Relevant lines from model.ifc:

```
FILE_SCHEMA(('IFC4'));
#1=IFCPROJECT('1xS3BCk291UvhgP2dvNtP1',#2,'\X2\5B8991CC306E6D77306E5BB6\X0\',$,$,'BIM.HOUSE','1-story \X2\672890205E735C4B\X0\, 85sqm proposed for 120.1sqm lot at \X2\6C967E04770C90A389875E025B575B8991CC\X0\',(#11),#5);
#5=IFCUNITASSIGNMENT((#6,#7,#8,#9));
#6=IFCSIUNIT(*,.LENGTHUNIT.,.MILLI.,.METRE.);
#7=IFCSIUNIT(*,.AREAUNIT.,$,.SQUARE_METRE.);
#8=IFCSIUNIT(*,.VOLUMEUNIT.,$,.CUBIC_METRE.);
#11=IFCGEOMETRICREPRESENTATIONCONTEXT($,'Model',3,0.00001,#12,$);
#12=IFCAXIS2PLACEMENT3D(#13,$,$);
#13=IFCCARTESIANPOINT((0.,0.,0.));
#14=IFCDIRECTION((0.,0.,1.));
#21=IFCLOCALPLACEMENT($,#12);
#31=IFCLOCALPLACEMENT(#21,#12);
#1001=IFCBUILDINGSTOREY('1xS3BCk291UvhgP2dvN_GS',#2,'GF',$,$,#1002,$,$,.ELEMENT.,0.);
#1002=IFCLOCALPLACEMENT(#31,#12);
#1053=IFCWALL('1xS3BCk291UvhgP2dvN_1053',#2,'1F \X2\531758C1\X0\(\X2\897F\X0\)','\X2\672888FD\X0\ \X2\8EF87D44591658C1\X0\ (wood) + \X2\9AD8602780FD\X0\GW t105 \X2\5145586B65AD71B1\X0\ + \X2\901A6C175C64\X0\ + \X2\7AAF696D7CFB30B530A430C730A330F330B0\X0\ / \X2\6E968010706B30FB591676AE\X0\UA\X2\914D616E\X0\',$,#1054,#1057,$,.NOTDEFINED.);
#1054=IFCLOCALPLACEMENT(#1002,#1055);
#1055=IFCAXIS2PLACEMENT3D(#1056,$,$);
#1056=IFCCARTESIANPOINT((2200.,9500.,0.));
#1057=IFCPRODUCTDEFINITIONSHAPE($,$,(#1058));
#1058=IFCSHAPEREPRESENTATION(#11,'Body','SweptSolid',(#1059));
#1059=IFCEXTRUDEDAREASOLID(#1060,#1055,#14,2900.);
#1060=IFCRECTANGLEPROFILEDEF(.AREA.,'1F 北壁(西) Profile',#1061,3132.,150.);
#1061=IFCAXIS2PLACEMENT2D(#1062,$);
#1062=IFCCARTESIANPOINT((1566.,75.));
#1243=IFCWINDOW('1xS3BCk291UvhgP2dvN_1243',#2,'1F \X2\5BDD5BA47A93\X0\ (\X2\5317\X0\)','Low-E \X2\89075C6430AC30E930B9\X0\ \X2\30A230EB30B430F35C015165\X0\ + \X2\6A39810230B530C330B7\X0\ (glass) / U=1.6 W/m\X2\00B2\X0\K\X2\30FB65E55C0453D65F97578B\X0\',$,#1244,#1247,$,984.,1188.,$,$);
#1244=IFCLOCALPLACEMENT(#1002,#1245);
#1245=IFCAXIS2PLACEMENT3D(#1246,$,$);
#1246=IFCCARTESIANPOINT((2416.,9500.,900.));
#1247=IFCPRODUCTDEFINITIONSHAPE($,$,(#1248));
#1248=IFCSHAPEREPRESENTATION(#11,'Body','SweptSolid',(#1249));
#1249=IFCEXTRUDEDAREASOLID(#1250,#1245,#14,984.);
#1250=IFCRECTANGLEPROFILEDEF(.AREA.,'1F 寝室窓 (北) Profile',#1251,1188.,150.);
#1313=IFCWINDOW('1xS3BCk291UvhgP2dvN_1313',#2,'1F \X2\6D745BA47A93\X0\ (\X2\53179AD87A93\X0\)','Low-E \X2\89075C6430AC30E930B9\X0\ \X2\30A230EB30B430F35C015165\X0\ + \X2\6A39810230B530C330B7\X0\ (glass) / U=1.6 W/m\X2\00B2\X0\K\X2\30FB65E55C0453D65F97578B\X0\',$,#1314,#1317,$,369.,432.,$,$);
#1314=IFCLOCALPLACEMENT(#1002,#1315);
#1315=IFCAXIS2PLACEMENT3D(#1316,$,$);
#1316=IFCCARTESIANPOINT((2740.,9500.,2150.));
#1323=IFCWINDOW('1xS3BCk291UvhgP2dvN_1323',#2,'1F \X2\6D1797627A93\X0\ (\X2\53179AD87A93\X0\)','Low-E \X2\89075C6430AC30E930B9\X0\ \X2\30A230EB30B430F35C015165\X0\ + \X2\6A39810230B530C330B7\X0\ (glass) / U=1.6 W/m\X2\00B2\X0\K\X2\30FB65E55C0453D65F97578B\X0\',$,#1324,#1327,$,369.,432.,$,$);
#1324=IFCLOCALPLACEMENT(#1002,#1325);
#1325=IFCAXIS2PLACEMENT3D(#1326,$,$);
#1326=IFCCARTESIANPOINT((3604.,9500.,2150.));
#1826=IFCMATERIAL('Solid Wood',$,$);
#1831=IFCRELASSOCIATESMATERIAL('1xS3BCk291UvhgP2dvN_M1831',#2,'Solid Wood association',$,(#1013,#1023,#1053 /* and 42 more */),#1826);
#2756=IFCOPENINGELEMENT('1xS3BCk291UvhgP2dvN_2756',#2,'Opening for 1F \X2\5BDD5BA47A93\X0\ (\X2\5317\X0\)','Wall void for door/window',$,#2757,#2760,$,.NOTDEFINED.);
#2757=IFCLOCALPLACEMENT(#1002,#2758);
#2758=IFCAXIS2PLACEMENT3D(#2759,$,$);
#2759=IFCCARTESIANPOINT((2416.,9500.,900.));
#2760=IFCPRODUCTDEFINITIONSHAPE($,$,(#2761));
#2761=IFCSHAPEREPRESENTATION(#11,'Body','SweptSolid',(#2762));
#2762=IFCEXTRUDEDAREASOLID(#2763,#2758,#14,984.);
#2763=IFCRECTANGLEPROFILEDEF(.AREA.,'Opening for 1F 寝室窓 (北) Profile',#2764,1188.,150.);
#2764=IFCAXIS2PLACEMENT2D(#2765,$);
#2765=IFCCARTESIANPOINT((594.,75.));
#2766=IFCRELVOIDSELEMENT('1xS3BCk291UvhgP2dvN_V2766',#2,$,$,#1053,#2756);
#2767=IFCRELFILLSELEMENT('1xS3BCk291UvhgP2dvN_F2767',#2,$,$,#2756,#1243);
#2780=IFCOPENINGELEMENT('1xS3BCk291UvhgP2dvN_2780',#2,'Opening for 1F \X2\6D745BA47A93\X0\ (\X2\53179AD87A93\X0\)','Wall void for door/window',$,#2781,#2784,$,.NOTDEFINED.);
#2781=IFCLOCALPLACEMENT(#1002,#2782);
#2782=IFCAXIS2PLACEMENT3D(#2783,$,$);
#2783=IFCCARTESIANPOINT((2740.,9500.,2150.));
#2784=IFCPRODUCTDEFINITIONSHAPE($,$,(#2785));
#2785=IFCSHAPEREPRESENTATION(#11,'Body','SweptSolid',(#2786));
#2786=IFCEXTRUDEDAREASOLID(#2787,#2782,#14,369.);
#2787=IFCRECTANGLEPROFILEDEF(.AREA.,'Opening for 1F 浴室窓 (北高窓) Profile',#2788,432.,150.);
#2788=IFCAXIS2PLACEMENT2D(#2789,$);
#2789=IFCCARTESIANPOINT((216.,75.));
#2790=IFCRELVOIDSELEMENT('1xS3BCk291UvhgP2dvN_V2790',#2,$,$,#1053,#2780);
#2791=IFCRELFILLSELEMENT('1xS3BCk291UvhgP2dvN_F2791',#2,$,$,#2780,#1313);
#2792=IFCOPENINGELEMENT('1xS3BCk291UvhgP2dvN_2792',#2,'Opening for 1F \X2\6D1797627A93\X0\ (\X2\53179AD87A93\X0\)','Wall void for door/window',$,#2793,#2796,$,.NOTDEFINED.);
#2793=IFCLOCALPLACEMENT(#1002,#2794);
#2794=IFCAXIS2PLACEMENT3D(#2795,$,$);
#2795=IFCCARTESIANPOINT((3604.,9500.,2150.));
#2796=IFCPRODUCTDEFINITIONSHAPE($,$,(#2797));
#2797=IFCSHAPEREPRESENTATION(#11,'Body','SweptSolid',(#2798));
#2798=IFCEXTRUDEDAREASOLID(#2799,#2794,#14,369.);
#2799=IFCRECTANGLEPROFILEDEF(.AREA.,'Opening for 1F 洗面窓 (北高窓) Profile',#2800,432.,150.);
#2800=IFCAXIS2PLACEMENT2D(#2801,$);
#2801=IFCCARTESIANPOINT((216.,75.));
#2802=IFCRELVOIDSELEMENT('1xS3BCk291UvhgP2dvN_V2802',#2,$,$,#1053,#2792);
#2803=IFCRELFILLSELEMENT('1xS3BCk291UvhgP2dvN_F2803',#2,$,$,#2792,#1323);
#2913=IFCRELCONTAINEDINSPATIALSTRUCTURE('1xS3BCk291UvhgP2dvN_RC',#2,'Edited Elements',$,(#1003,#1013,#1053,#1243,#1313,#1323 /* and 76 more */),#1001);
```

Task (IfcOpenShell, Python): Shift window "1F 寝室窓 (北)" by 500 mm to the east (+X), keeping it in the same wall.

```python
import ifcopenshell
import ifcopenshell.api.geometry
import ifcopenshell.util.placement

model = ifcopenshell.open("model.ifc")

window = model.by_guid("1xS3BCk291UvhgP2dvN_1243")
opening = window.FillsVoids[0].RelatingOpeningElement
wall = opening.VoidsElements[0].RelatingBuildingElement

wall_matrix = ifcopenshell.util.placement.get_local_placement(wall.ObjectPlacement)
shift = wall_matrix[:3, 0] * 500.0
before = ifcopenshell.util.placement.get_local_placement(window.ObjectPlacement)[:3, 3].copy()

# The window is not placed relative to its opening, so move both.
for product in (opening, window):
    matrix = ifcopenshell.util.placement.get_local_placement(product.ObjectPlacement)
    matrix[:3, 3] += shift
    ifcopenshell.api.geometry.edit_object_placement(model, product=product, matrix=matrix, is_si=False)

after = ifcopenshell.util.placement.get_local_placement(window.ObjectPlacement)[:3, 3]
print("window moved by", (after - before).round(3) + 0.0)

model.write("model_v2.ifc")
```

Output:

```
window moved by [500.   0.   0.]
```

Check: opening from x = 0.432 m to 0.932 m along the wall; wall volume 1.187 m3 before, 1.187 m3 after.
